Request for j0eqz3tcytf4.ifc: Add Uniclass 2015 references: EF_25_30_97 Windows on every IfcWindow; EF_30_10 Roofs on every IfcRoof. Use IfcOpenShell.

First a look at what the model holds.

```python
import ifcopenshell

model = ifcopenshell.open("j0eqz3tcytf4.ifc")
print(model.schema)
print("classifications:", [c.Name for c in model.by_type("IfcClassification")])
for ifc_class in ("IfcDoor", "IfcRoof", "IfcStair", "IfcWall", "IfcWindow"):
    print(ifc_class, len(model.by_type(ifc_class)))
```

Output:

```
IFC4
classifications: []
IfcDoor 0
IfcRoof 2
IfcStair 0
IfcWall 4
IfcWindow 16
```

```python
import ifcopenshell
import ifcopenshell.api.classification

model = ifcopenshell.open("j0eqz3tcytf4.ifc")

system = ifcopenshell.api.classification.add_classification(model, classification="Uniclass 2015")

codes = {
    "IfcWindow": ("EF_25_30_97", "Windows"),
    "IfcRoof": ("EF_30_10", "Roofs"),
}
for ifc_class, (code, name) in codes.items():
    products = model.by_type(ifc_class)
    ifcopenshell.api.classification.add_reference(
        model, products=products, classification=system, identification=code, name=name
    )
    print(code, len(products))

model.write("j0eqz3tcytf4_v2.ifc")
```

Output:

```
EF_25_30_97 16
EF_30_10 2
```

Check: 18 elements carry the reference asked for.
